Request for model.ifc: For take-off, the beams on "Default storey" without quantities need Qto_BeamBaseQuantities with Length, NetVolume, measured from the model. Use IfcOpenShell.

First a look at what the model holds.

```python
import ifcopenshell
import ifcopenshell.util.element
import ifcopenshell.util.unit

model = ifcopenshell.open("model.ifc")
print(model.schema)
for unit_type in ("LENGTHUNIT", "AREAUNIT", "VOLUMEUNIT"):
    print(unit_type, ifcopenshell.util.unit.calculate_unit_scale(model, unit_type))
storey = next(s for s in model.by_type("IfcBuildingStorey") if s.Name == "Default storey")
beams = [e for e in ifcopenshell.util.element.get_decomposition(storey) if e.is_a("IfcBeam")]
for e in sorted(beams, key=lambda e: e.id()):
    print(e.id(), e.is_a(), e.Name, list(ifcopenshell.util.element.get_psets(e, qtos_only=True)), sep=" | ")
```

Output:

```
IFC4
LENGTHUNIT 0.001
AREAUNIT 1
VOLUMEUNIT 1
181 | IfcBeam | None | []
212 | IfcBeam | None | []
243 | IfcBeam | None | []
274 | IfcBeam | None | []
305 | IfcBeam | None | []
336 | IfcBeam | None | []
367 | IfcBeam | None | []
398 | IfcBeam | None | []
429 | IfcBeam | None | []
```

```python
import ifcopenshell
import ifcopenshell.api.pset
import ifcopenshell.geom
import ifcopenshell.util.element
import ifcopenshell.util.shape
import ifcopenshell.util.unit

model = ifcopenshell.open("model.ifc")
unit_scale = ifcopenshell.util.unit.calculate_unit_scale(model)
volume_scale = ifcopenshell.util.unit.calculate_unit_scale(model, "VOLUMEUNIT")
settings = ifcopenshell.geom.settings()

storey = next(s for s in model.by_type("IfcBuildingStorey") if s.Name == "Default storey")
beams = [e for e in ifcopenshell.util.element.get_decomposition(storey) if e.is_a("IfcBeam")]

for e in sorted(beams, key=lambda e: e.id()):
    if ifcopenshell.util.element.get_psets(e, qtos_only=True, should_inherit=False):
        continue
    # Geometry comes back in metres, in the element's own axes.
    shape = ifcopenshell.geom.create_shape(settings, e)
    values = {
        "Length": ifcopenshell.util.shape.get_max_xyz(shape.geometry) / unit_scale,
        "NetVolume": ifcopenshell.util.shape.get_volume(shape.geometry) / volume_scale,
    }
    qto = ifcopenshell.api.pset.add_qto(model, product=e, name="Qto_BeamBaseQuantities")
    ifcopenshell.api.pset.edit_qto(model, qto=qto, properties=values)
    print(e.id(), {k: round(v, 3) for k, v in values.items()})

model.write("model_edited.ifc")
```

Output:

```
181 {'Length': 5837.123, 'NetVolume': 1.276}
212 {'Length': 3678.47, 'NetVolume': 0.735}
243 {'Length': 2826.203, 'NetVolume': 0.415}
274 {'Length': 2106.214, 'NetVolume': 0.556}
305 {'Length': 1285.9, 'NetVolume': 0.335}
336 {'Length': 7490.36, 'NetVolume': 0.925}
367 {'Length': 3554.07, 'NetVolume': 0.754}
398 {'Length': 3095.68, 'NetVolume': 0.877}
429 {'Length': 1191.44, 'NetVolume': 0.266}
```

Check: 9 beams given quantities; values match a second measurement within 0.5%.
